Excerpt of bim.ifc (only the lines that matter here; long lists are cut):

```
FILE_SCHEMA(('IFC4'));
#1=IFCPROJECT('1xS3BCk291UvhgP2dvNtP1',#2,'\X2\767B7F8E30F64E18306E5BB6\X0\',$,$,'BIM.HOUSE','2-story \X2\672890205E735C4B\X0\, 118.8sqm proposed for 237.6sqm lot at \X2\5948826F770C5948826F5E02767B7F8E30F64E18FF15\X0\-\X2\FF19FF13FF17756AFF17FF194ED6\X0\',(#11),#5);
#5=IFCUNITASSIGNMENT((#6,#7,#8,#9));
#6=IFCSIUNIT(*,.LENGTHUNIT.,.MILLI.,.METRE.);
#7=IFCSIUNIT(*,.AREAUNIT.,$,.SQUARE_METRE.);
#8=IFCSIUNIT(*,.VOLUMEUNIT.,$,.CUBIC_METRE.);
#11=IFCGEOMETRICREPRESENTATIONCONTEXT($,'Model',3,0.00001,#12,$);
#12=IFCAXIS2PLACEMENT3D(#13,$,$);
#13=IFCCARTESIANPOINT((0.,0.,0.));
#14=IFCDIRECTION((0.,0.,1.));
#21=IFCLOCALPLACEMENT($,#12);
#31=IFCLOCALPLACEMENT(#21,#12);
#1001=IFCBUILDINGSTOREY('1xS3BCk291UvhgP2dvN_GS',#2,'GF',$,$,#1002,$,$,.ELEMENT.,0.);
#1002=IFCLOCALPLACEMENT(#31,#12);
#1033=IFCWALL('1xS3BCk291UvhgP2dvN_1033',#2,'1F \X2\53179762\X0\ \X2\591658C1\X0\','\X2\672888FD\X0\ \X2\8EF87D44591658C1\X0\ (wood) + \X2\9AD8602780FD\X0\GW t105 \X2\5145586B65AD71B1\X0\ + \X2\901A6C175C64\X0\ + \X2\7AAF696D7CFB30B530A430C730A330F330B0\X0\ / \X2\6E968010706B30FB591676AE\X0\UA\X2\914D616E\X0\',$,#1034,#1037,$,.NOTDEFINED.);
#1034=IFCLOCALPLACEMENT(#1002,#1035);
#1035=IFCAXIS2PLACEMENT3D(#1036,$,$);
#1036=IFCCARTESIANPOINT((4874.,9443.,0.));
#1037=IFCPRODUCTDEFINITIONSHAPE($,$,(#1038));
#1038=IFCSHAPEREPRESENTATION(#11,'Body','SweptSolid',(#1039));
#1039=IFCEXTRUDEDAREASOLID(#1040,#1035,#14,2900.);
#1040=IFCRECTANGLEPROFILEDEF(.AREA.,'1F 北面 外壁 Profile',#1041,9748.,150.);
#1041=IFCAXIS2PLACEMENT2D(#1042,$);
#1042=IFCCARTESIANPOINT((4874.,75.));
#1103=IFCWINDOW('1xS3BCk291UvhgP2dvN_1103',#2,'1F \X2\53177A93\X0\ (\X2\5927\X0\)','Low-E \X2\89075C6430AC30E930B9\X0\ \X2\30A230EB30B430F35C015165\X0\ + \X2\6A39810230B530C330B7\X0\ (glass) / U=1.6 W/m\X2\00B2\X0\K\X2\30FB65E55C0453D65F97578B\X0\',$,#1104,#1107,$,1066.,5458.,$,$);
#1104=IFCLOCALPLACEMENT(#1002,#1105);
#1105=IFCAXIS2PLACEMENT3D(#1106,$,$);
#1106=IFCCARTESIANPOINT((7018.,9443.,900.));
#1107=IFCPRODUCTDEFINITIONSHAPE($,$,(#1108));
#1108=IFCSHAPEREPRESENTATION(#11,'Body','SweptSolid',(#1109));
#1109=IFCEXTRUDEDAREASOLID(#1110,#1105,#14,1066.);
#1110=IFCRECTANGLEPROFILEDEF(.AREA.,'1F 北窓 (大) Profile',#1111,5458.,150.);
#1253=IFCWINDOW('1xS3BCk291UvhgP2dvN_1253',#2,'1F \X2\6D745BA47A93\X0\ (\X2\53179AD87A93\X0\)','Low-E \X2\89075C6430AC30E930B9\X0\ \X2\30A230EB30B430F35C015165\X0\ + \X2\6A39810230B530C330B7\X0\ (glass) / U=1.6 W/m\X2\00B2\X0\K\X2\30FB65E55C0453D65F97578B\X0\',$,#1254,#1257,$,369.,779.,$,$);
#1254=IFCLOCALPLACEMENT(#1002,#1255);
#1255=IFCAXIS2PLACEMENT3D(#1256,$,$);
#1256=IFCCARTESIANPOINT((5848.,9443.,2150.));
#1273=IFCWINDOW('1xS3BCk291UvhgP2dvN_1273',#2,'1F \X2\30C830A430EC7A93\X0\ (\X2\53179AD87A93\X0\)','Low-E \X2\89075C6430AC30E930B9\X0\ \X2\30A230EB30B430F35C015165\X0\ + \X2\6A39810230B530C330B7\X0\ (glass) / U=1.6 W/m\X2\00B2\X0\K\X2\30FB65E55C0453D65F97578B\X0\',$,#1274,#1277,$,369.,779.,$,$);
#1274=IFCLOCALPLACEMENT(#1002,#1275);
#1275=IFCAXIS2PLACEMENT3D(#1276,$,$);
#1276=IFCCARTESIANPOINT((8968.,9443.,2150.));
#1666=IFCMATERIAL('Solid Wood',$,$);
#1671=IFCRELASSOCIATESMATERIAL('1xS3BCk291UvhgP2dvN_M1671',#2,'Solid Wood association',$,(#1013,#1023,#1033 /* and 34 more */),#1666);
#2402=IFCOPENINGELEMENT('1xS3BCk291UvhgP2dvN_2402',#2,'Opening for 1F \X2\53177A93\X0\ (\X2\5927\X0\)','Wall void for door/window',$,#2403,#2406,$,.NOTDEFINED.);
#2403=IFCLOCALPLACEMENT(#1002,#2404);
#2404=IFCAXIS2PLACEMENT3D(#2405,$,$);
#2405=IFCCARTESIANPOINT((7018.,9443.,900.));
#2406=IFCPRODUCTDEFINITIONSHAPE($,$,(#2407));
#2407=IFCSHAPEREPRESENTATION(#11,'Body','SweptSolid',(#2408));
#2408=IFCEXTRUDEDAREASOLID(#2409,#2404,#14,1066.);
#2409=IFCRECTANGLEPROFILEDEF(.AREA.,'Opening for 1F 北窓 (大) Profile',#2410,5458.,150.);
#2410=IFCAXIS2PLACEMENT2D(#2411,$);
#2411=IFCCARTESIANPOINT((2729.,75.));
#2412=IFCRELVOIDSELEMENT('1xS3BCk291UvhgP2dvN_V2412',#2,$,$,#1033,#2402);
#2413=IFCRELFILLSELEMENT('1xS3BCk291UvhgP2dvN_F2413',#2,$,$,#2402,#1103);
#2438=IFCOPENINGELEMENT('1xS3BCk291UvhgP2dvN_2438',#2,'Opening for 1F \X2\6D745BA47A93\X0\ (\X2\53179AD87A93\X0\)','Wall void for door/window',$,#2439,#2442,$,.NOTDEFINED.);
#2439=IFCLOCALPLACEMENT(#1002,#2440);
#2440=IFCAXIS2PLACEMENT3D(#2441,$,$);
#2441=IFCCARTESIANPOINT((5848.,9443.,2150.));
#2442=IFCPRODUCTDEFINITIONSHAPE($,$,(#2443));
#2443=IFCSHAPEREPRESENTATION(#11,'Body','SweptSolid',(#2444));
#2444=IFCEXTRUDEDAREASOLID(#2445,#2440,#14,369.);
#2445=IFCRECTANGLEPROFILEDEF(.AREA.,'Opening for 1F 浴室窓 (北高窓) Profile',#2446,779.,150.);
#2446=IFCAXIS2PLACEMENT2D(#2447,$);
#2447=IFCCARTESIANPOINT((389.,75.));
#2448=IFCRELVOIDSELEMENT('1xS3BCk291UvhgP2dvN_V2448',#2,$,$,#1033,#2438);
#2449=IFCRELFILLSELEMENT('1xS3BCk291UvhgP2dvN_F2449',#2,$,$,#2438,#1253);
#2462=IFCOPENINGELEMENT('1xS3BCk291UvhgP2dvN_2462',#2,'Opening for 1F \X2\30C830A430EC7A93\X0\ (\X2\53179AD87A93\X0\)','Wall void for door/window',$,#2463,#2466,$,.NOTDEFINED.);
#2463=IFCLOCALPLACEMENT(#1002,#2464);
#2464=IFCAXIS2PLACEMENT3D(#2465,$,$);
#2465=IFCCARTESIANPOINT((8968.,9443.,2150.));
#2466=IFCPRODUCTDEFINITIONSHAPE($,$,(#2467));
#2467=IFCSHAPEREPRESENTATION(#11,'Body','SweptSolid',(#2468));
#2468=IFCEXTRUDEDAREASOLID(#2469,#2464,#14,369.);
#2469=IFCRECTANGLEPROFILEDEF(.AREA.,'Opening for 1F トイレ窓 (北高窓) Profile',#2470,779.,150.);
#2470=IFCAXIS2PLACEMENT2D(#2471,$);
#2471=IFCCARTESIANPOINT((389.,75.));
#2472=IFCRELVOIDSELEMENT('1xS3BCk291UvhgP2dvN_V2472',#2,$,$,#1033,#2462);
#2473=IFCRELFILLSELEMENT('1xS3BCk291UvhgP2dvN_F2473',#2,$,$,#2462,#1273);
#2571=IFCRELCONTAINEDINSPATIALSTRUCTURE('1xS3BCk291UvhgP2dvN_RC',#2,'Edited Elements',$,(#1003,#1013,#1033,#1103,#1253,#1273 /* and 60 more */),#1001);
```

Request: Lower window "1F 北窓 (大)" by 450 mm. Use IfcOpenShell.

```python
import numpy as np
import ifcopenshell
import ifcopenshell.api.geometry
import ifcopenshell.util.placement
import ifcopenshell.util.unit

model = ifcopenshell.open("bim.ifc")
unit_scale = ifcopenshell.util.unit.calculate_unit_scale(model)

window = model.by_guid("1xS3BCk291UvhgP2dvN_1103")
opening = window.FillsVoids[0].RelatingOpeningElement
dz = -0.45 / unit_scale

shift = np.array([0.0, 0.0, dz])
# The window is not placed relative to its opening, so move both.
for product in (opening, window):
    matrix = ifcopenshell.util.placement.get_local_placement(product.ObjectPlacement)
    matrix[:3, 3] += shift
    ifcopenshell.api.geometry.edit_object_placement(model, product=product, matrix=matrix, is_si=False)

print(f"moved by {dz * unit_scale:+.3f} m")

model.write("bim_v2.ifc")
```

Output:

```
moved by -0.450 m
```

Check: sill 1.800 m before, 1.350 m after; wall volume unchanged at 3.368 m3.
